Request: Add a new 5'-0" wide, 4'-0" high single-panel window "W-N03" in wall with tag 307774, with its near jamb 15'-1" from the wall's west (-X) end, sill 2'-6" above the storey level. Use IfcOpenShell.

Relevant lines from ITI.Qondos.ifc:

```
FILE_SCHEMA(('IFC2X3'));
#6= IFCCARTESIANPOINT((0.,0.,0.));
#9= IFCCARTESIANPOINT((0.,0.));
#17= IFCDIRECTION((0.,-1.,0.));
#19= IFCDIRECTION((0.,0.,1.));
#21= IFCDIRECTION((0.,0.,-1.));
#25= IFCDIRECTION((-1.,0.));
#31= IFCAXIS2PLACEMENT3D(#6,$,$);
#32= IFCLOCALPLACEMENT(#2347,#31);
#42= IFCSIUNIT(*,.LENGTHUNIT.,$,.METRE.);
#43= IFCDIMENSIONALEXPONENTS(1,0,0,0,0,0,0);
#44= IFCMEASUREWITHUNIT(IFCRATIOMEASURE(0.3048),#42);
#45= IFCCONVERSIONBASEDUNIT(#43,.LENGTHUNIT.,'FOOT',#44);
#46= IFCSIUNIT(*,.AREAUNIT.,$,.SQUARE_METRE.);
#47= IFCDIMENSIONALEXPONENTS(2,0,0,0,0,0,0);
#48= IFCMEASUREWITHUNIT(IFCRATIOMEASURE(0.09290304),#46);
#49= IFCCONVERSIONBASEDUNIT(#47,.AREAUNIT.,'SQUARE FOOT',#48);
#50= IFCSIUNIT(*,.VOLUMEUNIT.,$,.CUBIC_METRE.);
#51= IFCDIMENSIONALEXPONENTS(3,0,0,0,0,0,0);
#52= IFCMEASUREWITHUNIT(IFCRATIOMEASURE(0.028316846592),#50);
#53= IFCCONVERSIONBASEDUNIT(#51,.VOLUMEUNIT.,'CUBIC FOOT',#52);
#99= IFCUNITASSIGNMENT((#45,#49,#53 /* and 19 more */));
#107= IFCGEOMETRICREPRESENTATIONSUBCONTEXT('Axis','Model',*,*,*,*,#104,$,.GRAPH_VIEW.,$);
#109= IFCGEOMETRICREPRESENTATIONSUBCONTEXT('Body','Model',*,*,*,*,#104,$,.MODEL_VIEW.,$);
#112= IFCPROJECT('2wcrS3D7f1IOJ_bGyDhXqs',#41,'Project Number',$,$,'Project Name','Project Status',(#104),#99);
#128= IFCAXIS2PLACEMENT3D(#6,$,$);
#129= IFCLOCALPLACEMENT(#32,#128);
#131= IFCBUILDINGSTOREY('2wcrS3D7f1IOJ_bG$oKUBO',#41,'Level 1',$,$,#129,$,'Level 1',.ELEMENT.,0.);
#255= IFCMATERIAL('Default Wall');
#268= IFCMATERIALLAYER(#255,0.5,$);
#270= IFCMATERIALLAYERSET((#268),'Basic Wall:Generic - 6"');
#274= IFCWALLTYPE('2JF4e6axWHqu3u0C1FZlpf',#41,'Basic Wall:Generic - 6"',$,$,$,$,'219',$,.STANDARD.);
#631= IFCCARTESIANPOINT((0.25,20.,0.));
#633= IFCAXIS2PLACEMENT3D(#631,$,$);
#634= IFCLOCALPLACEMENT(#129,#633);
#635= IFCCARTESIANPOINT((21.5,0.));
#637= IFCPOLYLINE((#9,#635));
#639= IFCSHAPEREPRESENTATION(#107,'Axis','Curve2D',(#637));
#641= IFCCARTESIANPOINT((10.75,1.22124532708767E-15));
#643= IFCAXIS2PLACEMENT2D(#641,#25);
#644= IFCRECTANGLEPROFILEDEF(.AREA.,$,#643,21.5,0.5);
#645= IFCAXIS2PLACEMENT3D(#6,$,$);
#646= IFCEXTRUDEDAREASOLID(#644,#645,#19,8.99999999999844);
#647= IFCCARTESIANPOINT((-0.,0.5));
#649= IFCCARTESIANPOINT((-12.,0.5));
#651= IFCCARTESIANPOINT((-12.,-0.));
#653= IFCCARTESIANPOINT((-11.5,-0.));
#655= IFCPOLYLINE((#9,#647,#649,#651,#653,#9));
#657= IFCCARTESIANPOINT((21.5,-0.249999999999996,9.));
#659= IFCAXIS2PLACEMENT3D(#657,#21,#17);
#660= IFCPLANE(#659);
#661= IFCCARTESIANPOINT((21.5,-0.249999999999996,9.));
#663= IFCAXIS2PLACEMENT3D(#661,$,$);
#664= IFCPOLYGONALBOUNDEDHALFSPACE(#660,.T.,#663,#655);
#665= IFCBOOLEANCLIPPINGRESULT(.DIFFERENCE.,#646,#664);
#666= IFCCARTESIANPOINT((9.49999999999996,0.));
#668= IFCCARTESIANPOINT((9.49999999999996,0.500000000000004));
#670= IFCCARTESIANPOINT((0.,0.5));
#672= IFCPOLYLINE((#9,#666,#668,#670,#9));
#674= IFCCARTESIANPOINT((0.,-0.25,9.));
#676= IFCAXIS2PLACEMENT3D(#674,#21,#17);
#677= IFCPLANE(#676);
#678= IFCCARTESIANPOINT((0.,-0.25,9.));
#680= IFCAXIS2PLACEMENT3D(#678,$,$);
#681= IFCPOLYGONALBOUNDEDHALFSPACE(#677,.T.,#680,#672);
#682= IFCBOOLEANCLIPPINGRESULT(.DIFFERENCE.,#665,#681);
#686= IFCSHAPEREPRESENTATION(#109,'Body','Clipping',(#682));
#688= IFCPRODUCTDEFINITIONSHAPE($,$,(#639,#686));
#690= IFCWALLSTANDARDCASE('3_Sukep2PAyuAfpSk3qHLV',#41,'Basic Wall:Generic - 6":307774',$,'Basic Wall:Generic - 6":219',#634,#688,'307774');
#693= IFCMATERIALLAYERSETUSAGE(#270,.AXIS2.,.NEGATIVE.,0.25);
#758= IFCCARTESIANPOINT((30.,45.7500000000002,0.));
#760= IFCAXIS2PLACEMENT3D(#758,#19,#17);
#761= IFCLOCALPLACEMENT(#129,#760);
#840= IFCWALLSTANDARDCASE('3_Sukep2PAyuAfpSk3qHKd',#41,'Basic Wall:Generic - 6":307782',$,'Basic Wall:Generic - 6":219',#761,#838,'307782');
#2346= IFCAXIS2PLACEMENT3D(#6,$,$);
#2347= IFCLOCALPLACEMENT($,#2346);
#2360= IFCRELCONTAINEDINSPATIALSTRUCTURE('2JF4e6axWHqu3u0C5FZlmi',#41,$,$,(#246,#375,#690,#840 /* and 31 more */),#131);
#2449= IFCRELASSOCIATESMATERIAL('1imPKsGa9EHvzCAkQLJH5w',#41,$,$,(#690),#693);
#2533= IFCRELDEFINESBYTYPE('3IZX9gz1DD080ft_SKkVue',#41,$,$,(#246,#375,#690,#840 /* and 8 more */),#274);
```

```python
import numpy as np
import ifcopenshell
import ifcopenshell.api.feature
import ifcopenshell.api.geometry
import ifcopenshell.api.root
import ifcopenshell.api.spatial
import ifcopenshell.api.type
import ifcopenshell.geom
import ifcopenshell.util.element
import ifcopenshell.util.placement
import ifcopenshell.util.representation
import ifcopenshell.util.shape
import ifcopenshell.util.unit

model = ifcopenshell.open("ITI.Qondos.ifc")
unit_scale = ifcopenshell.util.unit.calculate_unit_scale(model)
settings = ifcopenshell.geom.settings()


def volume(element):
    """Net volume in cubic metres, openings subtracted."""
    shape = ifcopenshell.geom.create_shape(settings, element)
    return ifcopenshell.util.shape.get_volume(shape.geometry)


wall = model.by_guid("3_Sukep2PAyuAfpSk3qHLV")
storey = ifcopenshell.util.element.get_container(wall, ifc_class="IfcBuildingStorey")
context = ifcopenshell.util.representation.get_context(model, "Model", "Body", "MODEL_VIEW")
before = volume(wall)

width, height, from_end, sill = 1.524, 1.2192, 4.5974, 0.762  # metres

# The wall runs along its own X axis, and the end named is its -X end.
wall_shape = ifcopenshell.geom.create_shape(settings, wall)
x, y, z = ifcopenshell.util.shape.get_vertices(wall_shape.geometry).T
start = x.min() + from_end
face, thickness = float(y.min()), float(y.max() - y.min())
wall_matrix = ifcopenshell.util.placement.get_local_placement(wall.ObjectPlacement)
level = ifcopenshell.util.placement.get_local_placement(storey.ObjectPlacement)[2, 3]


def in_wall(x, y):
    """Placement at x, y metres in the wall's axes, at sill height."""
    matrix = wall_matrix.copy()
    matrix[:, 3] = wall_matrix @ np.array([x / unit_scale, y / unit_scale, 0.0, 1.0])
    matrix[2, 3] = level + sill / unit_scale
    return matrix


# Opening: a box that overshoots both wall faces by 50 mm.
opening = ifcopenshell.api.root.create_entity(model, ifc_class="IfcOpeningElement")
box = ifcopenshell.api.geometry.add_wall_representation(
    model, context=context, length=width, height=height, thickness=thickness + 0.1
)
ifcopenshell.api.geometry.assign_representation(model, product=opening, representation=box)
ifcopenshell.api.geometry.edit_object_placement(model, product=opening, matrix=in_wall(start, face - 0.05), is_si=False)
ifcopenshell.api.feature.add_feature(model, feature=opening, element=wall)

window = ifcopenshell.api.root.create_entity(model, ifc_class="IfcWindow", name="W-N03")
window.OverallWidth, window.OverallHeight = width / unit_scale, height / unit_scale
body = ifcopenshell.api.geometry.add_window_representation(
    model,
    context=context,
    overall_width=window.OverallWidth,
    overall_height=window.OverallHeight,
    partition_type="SINGLE_PANEL",
)
ifcopenshell.api.geometry.assign_representation(model, product=window, representation=body)
ifcopenshell.api.spatial.assign_container(model, products=[window], relating_structure=storey)
fills = ifcopenshell.api.feature.add_filling(model, opening=opening, element=window)
fills.OwnerHistory = window.OwnerHistory  # required in IFC2X3

# IFC2X3 keeps the operation on the window style.
style = ifcopenshell.api.root.create_entity(model, ifc_class="IfcWindowStyle", name="W-N03")
style.OperationType, style.ConstructionType = "SINGLE_PANEL", "NOTDEFINED"
style.ParameterTakesPrecedence = style.Sizeable = False
ifcopenshell.api.type.assign_type(model, related_objects=[window], relating_type=style)

# Centre the window in the wall's thickness.
ifcopenshell.api.geometry.edit_object_placement(model, product=window, matrix=in_wall(start, face), is_si=False)
window_shape = ifcopenshell.geom.create_shape(settings, window)
depth = ifcopenshell.util.shape.get_vertices(window_shape.geometry)[:, 1]
offset = face + thickness / 2 - (depth.min() + depth.max()) / 2
ifcopenshell.api.geometry.edit_object_placement(model, product=window, matrix=in_wall(start, offset), is_si=False)

after = volume(wall)

print(f"wall volume {before:.3f} -> {after:.3f} m3")

model.write("ITI.Qondos_rev.ifc")
```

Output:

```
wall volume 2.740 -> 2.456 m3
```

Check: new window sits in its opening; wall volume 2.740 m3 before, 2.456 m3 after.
